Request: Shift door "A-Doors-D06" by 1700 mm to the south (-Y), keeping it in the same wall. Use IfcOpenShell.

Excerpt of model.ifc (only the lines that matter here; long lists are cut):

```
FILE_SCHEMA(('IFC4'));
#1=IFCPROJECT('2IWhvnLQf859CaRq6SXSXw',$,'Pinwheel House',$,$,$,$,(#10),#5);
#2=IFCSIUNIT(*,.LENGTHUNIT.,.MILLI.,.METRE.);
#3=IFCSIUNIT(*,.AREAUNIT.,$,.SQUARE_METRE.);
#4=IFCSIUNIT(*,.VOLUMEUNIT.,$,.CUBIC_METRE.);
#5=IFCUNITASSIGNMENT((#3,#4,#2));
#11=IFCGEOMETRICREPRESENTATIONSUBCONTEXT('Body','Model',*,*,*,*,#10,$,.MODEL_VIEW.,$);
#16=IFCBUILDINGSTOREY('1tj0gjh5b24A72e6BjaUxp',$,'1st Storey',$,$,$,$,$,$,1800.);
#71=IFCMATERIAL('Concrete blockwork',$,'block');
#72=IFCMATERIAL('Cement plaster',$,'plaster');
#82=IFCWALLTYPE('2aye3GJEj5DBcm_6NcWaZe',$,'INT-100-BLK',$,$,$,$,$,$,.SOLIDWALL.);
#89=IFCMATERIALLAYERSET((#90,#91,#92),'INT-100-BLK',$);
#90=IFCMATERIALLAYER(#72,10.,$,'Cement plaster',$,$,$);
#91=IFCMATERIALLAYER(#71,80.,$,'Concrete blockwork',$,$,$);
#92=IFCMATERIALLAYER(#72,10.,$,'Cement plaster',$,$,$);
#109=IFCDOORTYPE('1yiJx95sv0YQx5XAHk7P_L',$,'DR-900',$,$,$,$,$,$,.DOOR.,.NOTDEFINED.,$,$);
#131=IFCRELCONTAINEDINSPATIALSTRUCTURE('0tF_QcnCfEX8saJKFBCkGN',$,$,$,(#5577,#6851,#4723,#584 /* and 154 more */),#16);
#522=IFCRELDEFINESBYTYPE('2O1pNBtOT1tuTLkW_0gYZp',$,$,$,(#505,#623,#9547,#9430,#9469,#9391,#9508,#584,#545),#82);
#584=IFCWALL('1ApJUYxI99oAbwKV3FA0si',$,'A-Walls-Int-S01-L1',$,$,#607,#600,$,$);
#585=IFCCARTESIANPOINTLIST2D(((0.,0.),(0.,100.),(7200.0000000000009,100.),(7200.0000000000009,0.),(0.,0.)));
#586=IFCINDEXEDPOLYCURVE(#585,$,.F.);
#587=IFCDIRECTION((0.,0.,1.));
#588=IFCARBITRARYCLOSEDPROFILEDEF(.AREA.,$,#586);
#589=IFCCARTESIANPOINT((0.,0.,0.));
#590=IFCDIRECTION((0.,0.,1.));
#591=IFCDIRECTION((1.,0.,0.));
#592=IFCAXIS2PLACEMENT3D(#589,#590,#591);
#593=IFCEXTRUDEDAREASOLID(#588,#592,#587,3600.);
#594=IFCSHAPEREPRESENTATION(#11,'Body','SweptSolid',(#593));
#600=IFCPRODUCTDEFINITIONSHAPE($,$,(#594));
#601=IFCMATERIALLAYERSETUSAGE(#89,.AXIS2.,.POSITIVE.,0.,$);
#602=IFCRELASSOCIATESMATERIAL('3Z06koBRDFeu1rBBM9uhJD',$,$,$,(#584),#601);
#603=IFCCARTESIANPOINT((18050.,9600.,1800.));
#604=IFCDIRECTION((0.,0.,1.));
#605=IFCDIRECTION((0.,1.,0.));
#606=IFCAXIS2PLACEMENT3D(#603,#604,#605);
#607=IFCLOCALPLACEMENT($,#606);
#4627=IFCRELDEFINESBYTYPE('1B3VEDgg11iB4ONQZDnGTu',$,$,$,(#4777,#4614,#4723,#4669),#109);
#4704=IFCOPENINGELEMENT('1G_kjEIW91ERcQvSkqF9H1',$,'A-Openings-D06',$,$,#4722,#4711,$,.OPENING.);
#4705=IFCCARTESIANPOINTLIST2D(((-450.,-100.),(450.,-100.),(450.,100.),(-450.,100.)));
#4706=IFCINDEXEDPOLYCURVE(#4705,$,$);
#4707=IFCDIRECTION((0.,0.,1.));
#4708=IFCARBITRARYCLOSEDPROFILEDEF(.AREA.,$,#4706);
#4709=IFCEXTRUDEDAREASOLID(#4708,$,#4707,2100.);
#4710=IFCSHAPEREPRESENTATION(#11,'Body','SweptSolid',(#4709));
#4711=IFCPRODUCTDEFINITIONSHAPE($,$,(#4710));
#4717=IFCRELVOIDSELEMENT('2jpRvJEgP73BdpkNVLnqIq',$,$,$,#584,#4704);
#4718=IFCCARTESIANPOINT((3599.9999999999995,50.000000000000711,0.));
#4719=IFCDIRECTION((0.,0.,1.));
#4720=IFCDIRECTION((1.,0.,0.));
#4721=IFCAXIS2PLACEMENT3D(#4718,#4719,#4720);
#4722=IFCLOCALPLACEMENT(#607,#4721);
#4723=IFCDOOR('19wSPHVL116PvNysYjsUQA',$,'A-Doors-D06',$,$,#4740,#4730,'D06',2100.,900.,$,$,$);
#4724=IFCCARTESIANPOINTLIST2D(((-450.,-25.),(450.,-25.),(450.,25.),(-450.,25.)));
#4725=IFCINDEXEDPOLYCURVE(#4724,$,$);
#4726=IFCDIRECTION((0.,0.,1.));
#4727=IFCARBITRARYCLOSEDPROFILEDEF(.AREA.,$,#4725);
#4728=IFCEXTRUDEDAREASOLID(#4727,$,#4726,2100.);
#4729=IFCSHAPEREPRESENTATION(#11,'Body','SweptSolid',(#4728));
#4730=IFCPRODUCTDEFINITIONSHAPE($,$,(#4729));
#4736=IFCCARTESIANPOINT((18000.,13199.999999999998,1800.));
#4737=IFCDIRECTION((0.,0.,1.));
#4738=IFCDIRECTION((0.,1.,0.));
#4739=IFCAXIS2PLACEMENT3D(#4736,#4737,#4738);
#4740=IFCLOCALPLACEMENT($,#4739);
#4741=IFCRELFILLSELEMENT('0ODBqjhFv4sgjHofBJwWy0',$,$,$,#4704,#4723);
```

```python
import ifcopenshell
import ifcopenshell.api.geometry
import ifcopenshell.util.placement

model = ifcopenshell.open("model.ifc")

door = model.by_guid("19wSPHVL116PvNysYjsUQA")
opening = door.FillsVoids[0].RelatingOpeningElement
wall = opening.VoidsElements[0].RelatingBuildingElement

wall_matrix = ifcopenshell.util.placement.get_local_placement(wall.ObjectPlacement)
shift = wall_matrix[:3, 0] * -1700.0
before = ifcopenshell.util.placement.get_local_placement(door.ObjectPlacement)[:3, 3].copy()

# The door is not placed relative to its opening, so move both.
for product in (opening, door):
    matrix = ifcopenshell.util.placement.get_local_placement(product.ObjectPlacement)
    matrix[:3, 3] += shift
    ifcopenshell.api.geometry.edit_object_placement(model, product=product, matrix=matrix, is_si=False)

after = ifcopenshell.util.placement.get_local_placement(door.ObjectPlacement)[:3, 3]
print("door moved by", (after - before).round(3) + 0.0)

model.write("model-out.ifc")
```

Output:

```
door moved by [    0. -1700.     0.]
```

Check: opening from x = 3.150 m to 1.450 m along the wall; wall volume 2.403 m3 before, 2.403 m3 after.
